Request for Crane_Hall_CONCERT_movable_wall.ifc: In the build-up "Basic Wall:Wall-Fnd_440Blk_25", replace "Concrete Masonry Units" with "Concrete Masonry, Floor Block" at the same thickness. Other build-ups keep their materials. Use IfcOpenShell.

First a look at what the model holds.

```python
import ifcopenshell
import ifcopenshell.util.element

model = ifcopenshell.open("Crane_Hall_CONCERT_movable_wall.ifc")
print(model.schema)
for layer_set in model.by_type("IfcMaterialLayerSet"):
    if layer_set.LayerSetName == "Basic Wall:Wall-Fnd_440Blk_25":
        for layer in layer_set.MaterialLayers:
            print(layer.id(), layer.Material and layer.Material.Name, layer.LayerThickness, sep=" | ")
        print(len(ifcopenshell.util.element.get_elements_by_material(model, layer_set)), "elements and types use it")
print(sorted(m.Name for m in model.by_type("IfcMaterial") if m.Name)[:60])
```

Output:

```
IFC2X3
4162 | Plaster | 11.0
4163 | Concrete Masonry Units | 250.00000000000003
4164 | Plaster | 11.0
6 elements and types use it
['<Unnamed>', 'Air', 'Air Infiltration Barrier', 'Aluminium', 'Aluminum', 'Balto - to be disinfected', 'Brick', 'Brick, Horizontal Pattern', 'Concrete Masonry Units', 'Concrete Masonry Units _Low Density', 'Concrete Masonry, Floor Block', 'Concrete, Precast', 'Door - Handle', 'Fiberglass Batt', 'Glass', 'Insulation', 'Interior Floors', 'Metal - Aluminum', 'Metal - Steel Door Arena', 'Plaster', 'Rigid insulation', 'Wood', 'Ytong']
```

```python
import ifcopenshell
import ifcopenshell.api.material

model = ifcopenshell.open("Crane_Hall_CONCERT_movable_wall.ifc")

layer_set = next(s for s in model.by_type("IfcMaterialLayerSet") if s.LayerSetName == "Basic Wall:Wall-Fnd_440Blk_25")
layer = next(l for l in layer_set.MaterialLayers if l.Material and l.Material.Name == "Concrete Masonry Units")
material = next(m for m in model.by_type("IfcMaterial") if m.Name == "Concrete Masonry, Floor Block")

# Point this one layer at the other material; renaming the old one would change it everywhere.
ifcopenshell.api.material.edit_layer(model, layer=layer, attributes={}, material=material)

print([l.Material.Name if l.Material else None for l in layer_set.MaterialLayers])

model.write("Crane_Hall_CONCERT_movable_wall_v2.ifc")
```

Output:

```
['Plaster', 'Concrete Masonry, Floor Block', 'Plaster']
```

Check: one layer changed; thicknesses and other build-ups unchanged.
